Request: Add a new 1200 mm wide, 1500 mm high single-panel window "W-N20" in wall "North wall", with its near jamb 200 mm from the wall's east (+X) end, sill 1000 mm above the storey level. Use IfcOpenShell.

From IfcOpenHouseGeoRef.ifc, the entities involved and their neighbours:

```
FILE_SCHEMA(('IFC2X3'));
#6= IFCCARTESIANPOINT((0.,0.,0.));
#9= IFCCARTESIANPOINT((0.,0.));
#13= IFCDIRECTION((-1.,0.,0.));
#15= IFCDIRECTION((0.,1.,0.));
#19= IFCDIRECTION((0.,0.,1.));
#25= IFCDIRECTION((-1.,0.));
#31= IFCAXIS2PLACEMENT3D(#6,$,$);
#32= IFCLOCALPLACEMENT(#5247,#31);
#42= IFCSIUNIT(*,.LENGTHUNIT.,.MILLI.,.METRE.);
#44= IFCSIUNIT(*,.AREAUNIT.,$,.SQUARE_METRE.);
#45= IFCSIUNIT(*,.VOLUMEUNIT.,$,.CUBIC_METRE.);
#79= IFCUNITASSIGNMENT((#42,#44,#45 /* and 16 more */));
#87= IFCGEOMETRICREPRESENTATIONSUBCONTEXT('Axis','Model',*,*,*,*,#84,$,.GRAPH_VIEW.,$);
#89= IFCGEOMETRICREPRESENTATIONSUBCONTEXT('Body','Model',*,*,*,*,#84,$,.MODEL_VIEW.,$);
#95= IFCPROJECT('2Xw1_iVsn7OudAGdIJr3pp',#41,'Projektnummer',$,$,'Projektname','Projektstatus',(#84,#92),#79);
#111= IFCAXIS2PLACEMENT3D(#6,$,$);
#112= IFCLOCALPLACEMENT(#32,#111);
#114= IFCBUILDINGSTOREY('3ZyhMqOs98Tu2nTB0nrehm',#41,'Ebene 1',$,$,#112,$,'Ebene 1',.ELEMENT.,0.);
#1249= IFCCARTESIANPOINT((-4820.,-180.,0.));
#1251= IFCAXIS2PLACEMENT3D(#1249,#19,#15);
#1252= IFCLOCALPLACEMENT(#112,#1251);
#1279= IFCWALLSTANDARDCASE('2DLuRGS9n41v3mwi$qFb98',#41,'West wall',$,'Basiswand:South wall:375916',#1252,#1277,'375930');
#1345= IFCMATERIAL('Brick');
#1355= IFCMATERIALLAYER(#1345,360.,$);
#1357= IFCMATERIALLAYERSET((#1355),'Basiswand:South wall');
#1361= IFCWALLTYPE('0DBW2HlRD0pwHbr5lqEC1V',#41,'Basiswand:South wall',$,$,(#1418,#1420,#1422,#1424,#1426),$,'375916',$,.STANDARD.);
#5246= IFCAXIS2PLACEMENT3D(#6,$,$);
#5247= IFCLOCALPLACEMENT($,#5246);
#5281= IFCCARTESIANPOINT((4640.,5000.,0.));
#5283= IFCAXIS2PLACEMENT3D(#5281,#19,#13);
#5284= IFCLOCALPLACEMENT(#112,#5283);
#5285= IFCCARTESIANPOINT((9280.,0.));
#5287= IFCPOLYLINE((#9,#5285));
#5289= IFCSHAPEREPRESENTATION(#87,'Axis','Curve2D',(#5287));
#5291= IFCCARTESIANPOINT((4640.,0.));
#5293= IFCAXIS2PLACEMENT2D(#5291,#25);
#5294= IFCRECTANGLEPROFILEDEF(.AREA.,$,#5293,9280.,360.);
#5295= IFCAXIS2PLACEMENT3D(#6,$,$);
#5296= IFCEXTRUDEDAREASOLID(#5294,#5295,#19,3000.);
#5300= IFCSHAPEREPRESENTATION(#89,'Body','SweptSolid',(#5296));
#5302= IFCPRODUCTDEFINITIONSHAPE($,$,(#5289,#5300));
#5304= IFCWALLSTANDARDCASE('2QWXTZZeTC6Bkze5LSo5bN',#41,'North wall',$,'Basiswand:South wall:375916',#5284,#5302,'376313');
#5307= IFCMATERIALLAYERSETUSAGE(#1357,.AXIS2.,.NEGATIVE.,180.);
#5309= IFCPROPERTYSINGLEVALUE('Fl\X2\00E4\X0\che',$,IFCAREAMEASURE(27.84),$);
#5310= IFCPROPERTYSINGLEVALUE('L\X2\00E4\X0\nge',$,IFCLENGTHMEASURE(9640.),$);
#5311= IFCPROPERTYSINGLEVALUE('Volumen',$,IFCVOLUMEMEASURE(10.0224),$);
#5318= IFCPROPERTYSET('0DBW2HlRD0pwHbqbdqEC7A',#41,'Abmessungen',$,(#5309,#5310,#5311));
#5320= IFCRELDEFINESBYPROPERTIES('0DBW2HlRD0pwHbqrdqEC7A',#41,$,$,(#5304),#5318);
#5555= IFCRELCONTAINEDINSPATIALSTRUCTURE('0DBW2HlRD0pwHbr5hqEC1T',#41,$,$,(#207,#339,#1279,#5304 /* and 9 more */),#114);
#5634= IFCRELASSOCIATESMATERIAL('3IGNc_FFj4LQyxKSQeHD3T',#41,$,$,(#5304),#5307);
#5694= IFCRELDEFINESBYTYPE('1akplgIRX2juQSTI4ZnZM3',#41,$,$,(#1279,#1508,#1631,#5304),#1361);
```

```python
import numpy as np
import ifcopenshell
import ifcopenshell.api.feature
import ifcopenshell.api.geometry
import ifcopenshell.api.pset
import ifcopenshell.api.root
import ifcopenshell.api.spatial
import ifcopenshell.api.type
import ifcopenshell.geom
import ifcopenshell.util.element
import ifcopenshell.util.placement
import ifcopenshell.util.representation
import ifcopenshell.util.shape
import ifcopenshell.util.unit

model = ifcopenshell.open("IfcOpenHouseGeoRef.ifc")
unit_scale = ifcopenshell.util.unit.calculate_unit_scale(model)
area_scale = ifcopenshell.util.unit.calculate_unit_scale(model, "AREAUNIT")
volume_scale = ifcopenshell.util.unit.calculate_unit_scale(model, "VOLUMEUNIT")
settings = ifcopenshell.geom.settings()


def volume(element):
    """Net volume in cubic metres, openings subtracted."""
    shape = ifcopenshell.geom.create_shape(settings, element)
    return ifcopenshell.util.shape.get_volume(shape.geometry)


wall = model.by_id(5304)
storey = ifcopenshell.util.element.get_container(wall, ifc_class="IfcBuildingStorey")
context = ifcopenshell.util.representation.get_context(model, "Model", "Body", "MODEL_VIEW")
before = volume(wall)

width, height, from_end, sill = 1.2, 1.5, 0.2, 1  # metres

# The wall runs along its own X axis, and the end named is its -X end.
wall_shape = ifcopenshell.geom.create_shape(settings, wall)
x, y, z = ifcopenshell.util.shape.get_vertices(wall_shape.geometry).T
start = x.min() + from_end
face, thickness = float(y.min()), float(y.max() - y.min())
wall_matrix = ifcopenshell.util.placement.get_local_placement(wall.ObjectPlacement)
level = ifcopenshell.util.placement.get_local_placement(storey.ObjectPlacement)[2, 3]


def in_wall(x, y):
    """Placement at x, y metres in the wall's axes, at sill height."""
    matrix = wall_matrix.copy()
    matrix[:, 3] = wall_matrix @ np.array([x / unit_scale, y / unit_scale, 0.0, 1.0])
    matrix[2, 3] = level + sill / unit_scale
    return matrix


# Opening: a box that overshoots both wall faces by 50 mm.
opening = ifcopenshell.api.root.create_entity(model, ifc_class="IfcOpeningElement")
box = ifcopenshell.api.geometry.add_wall_representation(
    model, context=context, length=width, height=height, thickness=thickness + 0.1
)
ifcopenshell.api.geometry.assign_representation(model, product=opening, representation=box)
ifcopenshell.api.geometry.edit_object_placement(model, product=opening, matrix=in_wall(start, face - 0.05), is_si=False)
ifcopenshell.api.feature.add_feature(model, feature=opening, element=wall)

window = ifcopenshell.api.root.create_entity(model, ifc_class="IfcWindow", name="W-N20")
window.OverallWidth, window.OverallHeight = width / unit_scale, height / unit_scale
body = ifcopenshell.api.geometry.add_window_representation(
    model,
    context=context,
    overall_width=window.OverallWidth,
    overall_height=window.OverallHeight,
    partition_type="SINGLE_PANEL",
)
ifcopenshell.api.geometry.assign_representation(model, product=window, representation=body)
ifcopenshell.api.spatial.assign_container(model, products=[window], relating_structure=storey)
fills = ifcopenshell.api.feature.add_filling(model, opening=opening, element=window)
fills.OwnerHistory = window.OwnerHistory  # required in IFC2X3

# IFC2X3 keeps the operation on the window style.
style = ifcopenshell.api.root.create_entity(model, ifc_class="IfcWindowStyle", name="W-N20")
style.OperationType, style.ConstructionType = "SINGLE_PANEL", "NOTDEFINED"
style.ParameterTakesPrecedence = style.Sizeable = False
ifcopenshell.api.type.assign_type(model, related_objects=[window], relating_type=style)

# Centre the window in the wall's thickness.
ifcopenshell.api.geometry.edit_object_placement(model, product=window, matrix=in_wall(start, face), is_si=False)
window_shape = ifcopenshell.geom.create_shape(settings, window)
depth = ifcopenshell.util.shape.get_vertices(window_shape.geometry)[:, 1]
offset = face + thickness / 2 - (depth.min() + depth.max()) / 2
ifcopenshell.api.geometry.edit_object_placement(model, product=window, matrix=in_wall(start, offset), is_si=False)

after = volume(wall)

# Update the wall's stored quantities.
pset = model.by_id(ifcopenshell.util.element.get_pset(wall, "Abmessungen", should_inherit=False)["id"])
ifcopenshell.api.pset.edit_pset(model, pset=pset, properties={
    "Fläche": model.create_entity("IfcAreaMeasure", after / thickness / area_scale),
    "Volumen": model.create_entity("IfcVolumeMeasure", after / volume_scale),
})

print(f"wall volume {before:.3f} -> {after:.3f} m3")

model.write("IfcOpenHouseGeoRef_rev.ifc")
```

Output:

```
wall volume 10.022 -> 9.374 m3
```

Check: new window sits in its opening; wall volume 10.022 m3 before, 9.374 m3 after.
